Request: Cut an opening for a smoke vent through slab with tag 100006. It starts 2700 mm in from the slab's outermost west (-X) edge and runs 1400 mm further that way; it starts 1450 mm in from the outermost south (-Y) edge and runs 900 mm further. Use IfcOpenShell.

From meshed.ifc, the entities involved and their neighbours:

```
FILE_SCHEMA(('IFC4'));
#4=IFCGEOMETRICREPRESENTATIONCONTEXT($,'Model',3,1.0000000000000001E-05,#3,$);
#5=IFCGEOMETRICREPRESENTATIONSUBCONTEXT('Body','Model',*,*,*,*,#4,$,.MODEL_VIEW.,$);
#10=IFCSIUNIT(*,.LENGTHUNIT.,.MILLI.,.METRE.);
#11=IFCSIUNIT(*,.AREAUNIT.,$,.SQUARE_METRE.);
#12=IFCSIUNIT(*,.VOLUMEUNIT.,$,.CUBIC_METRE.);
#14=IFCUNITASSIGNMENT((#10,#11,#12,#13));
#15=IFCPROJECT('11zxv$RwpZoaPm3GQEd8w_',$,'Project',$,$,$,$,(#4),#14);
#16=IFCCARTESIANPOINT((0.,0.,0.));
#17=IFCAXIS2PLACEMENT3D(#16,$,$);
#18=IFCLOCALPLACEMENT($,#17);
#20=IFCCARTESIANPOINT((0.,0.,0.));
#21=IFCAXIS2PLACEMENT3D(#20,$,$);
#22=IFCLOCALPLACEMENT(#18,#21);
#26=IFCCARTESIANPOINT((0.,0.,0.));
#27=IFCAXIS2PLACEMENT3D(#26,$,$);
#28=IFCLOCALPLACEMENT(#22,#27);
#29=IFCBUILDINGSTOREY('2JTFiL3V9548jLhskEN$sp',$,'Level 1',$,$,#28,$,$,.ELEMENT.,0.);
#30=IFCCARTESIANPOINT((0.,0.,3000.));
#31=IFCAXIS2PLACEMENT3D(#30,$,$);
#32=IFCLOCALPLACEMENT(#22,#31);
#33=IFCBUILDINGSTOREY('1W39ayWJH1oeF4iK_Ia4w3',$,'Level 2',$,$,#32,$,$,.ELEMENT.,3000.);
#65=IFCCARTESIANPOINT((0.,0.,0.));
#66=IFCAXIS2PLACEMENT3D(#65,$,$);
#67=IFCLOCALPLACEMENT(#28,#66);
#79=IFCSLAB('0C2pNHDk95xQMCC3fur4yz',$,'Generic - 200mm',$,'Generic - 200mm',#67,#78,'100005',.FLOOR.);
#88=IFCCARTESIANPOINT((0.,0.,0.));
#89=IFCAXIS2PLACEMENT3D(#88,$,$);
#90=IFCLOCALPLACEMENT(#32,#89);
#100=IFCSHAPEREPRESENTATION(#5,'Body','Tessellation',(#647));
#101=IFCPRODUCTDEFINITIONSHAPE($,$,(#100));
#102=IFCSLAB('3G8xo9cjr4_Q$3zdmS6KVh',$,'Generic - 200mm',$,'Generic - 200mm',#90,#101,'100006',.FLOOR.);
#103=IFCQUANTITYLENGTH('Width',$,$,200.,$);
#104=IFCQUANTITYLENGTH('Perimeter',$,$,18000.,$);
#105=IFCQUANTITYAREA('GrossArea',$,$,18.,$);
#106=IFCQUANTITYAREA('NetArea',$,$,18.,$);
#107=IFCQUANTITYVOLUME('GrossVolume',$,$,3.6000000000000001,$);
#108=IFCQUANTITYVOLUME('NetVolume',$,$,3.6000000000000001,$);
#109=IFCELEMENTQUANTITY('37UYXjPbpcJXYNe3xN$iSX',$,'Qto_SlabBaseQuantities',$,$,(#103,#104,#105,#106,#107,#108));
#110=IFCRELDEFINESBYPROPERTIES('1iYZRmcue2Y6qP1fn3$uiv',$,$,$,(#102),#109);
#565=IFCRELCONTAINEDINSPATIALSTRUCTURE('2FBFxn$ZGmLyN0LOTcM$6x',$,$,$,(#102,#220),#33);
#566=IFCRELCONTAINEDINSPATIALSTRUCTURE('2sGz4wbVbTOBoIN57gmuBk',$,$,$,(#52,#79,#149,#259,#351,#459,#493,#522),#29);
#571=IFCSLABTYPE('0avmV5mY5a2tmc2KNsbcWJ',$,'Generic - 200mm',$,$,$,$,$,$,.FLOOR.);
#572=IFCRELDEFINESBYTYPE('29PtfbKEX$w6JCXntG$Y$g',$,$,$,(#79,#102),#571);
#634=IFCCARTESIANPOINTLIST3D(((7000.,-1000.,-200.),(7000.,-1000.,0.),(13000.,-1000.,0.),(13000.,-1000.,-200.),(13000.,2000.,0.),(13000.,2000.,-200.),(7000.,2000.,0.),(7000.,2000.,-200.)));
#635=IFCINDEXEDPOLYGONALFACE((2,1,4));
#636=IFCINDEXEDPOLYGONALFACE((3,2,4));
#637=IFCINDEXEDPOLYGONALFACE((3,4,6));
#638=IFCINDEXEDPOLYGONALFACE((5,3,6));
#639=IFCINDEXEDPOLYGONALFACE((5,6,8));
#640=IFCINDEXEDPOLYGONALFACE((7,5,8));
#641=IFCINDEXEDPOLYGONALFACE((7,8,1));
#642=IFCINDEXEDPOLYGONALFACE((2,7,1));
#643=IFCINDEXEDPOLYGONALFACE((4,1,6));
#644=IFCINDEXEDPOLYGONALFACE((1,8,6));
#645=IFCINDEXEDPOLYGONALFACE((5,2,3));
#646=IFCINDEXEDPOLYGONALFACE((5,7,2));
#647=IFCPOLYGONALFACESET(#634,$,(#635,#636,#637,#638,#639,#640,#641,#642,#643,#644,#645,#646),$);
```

```python
import numpy as np
import ifcopenshell
import ifcopenshell.api.feature
import ifcopenshell.api.geometry
import ifcopenshell.api.pset
import ifcopenshell.api.root
import ifcopenshell.geom
import ifcopenshell.util.element
import ifcopenshell.util.placement
import ifcopenshell.util.representation
import ifcopenshell.util.shape
import ifcopenshell.util.unit

model = ifcopenshell.open("meshed.ifc")
unit_scale = ifcopenshell.util.unit.calculate_unit_scale(model)
area_scale = ifcopenshell.util.unit.calculate_unit_scale(model, "AREAUNIT")
volume_scale = ifcopenshell.util.unit.calculate_unit_scale(model, "VOLUMEUNIT")
settings = ifcopenshell.geom.settings()


def volume(element):
    """Net volume in cubic metres, openings subtracted."""
    shape = ifcopenshell.geom.create_shape(settings, element)
    return ifcopenshell.util.shape.get_volume(shape.geometry)


slab = model.by_guid("3G8xo9cjr4_Q$3zdmS6KVh")
before = volume(slab)

# Extent in the slab's own axes, in metres. The edges named are its -X and -Y sides.
slab_shape = ifcopenshell.geom.create_shape(settings, slab)
vertices = ifcopenshell.util.shape.get_vertices(slab_shape.geometry)
x_min, y_min, bottom = vertices.min(axis=0)
top = vertices[:, 2].max()

opening = ifcopenshell.api.root.create_entity(model, ifc_class="IfcOpeningElement", name="Smoke vent opening", predefined_type="OPENING")
context = ifcopenshell.util.representation.get_context(model, "Model", "Body", "MODEL_VIEW")
width, depth = 1.4, 0.9
outline = [(0.0, 0.0), (width, 0.0), (width, depth), (0.0, depth), (0.0, 0.0)]
# Overshoot both faces by 50 mm so the cut is clean.
shape = ifcopenshell.api.geometry.add_slab_representation(
    model, context=context, depth=top - bottom + 0.1, polyline=outline
)
ifcopenshell.api.geometry.assign_representation(model, product=opening, representation=shape)

matrix = ifcopenshell.util.placement.get_local_placement(slab.ObjectPlacement)
matrix[:, 3] = matrix @ np.append(np.array([x_min + 2.7, y_min + 1.45, bottom - 0.05]) / unit_scale, 1.0)
ifcopenshell.api.geometry.edit_object_placement(model, product=opening, matrix=matrix, is_si=False)
ifcopenshell.api.feature.add_feature(model, feature=opening, element=slab)

after = volume(slab)

# Update the slab's stored quantities.
qto = model.by_id(ifcopenshell.util.element.get_pset(slab, "Qto_SlabBaseQuantities", should_inherit=False)["id"])
ifcopenshell.api.pset.edit_qto(model, qto=qto, properties={
    "NetArea": after / (top - bottom) / area_scale,
    "NetVolume": after / volume_scale,
})

print(f"slab volume {before:.3f} -> {after:.3f} m3")

model.write("meshed_edited.ifc")
```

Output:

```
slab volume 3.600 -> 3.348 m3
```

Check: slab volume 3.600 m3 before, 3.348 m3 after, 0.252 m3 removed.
